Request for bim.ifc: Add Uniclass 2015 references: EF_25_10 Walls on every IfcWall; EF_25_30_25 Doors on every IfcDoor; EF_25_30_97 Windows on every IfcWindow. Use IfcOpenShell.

First a look at what the model holds.

```python
import ifcopenshell

model = ifcopenshell.open("bim.ifc")
print(model.schema)
print("classifications:", [c.Name for c in model.by_type("IfcClassification")])
for ifc_class in ("IfcDoor", "IfcRoof", "IfcStair", "IfcWall", "IfcWindow"):
    print(ifc_class, len(model.by_type(ifc_class)))
```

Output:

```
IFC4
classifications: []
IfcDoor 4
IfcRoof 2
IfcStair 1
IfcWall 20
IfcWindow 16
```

```python
import ifcopenshell
import ifcopenshell.api.classification

model = ifcopenshell.open("bim.ifc")

system = ifcopenshell.api.classification.add_classification(model, classification="Uniclass 2015")

codes = {
    "IfcWall": ("EF_25_10", "Walls"),
    "IfcDoor": ("EF_25_30_25", "Doors"),
    "IfcWindow": ("EF_25_30_97", "Windows"),
}
for ifc_class, (code, name) in codes.items():
    products = model.by_type(ifc_class)
    ifcopenshell.api.classification.add_reference(
        model, products=products, classification=system, identification=code, name=name
    )
    print(code, len(products))

model.write("bim_v2.ifc")
```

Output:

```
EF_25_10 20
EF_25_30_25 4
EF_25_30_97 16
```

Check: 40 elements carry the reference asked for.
